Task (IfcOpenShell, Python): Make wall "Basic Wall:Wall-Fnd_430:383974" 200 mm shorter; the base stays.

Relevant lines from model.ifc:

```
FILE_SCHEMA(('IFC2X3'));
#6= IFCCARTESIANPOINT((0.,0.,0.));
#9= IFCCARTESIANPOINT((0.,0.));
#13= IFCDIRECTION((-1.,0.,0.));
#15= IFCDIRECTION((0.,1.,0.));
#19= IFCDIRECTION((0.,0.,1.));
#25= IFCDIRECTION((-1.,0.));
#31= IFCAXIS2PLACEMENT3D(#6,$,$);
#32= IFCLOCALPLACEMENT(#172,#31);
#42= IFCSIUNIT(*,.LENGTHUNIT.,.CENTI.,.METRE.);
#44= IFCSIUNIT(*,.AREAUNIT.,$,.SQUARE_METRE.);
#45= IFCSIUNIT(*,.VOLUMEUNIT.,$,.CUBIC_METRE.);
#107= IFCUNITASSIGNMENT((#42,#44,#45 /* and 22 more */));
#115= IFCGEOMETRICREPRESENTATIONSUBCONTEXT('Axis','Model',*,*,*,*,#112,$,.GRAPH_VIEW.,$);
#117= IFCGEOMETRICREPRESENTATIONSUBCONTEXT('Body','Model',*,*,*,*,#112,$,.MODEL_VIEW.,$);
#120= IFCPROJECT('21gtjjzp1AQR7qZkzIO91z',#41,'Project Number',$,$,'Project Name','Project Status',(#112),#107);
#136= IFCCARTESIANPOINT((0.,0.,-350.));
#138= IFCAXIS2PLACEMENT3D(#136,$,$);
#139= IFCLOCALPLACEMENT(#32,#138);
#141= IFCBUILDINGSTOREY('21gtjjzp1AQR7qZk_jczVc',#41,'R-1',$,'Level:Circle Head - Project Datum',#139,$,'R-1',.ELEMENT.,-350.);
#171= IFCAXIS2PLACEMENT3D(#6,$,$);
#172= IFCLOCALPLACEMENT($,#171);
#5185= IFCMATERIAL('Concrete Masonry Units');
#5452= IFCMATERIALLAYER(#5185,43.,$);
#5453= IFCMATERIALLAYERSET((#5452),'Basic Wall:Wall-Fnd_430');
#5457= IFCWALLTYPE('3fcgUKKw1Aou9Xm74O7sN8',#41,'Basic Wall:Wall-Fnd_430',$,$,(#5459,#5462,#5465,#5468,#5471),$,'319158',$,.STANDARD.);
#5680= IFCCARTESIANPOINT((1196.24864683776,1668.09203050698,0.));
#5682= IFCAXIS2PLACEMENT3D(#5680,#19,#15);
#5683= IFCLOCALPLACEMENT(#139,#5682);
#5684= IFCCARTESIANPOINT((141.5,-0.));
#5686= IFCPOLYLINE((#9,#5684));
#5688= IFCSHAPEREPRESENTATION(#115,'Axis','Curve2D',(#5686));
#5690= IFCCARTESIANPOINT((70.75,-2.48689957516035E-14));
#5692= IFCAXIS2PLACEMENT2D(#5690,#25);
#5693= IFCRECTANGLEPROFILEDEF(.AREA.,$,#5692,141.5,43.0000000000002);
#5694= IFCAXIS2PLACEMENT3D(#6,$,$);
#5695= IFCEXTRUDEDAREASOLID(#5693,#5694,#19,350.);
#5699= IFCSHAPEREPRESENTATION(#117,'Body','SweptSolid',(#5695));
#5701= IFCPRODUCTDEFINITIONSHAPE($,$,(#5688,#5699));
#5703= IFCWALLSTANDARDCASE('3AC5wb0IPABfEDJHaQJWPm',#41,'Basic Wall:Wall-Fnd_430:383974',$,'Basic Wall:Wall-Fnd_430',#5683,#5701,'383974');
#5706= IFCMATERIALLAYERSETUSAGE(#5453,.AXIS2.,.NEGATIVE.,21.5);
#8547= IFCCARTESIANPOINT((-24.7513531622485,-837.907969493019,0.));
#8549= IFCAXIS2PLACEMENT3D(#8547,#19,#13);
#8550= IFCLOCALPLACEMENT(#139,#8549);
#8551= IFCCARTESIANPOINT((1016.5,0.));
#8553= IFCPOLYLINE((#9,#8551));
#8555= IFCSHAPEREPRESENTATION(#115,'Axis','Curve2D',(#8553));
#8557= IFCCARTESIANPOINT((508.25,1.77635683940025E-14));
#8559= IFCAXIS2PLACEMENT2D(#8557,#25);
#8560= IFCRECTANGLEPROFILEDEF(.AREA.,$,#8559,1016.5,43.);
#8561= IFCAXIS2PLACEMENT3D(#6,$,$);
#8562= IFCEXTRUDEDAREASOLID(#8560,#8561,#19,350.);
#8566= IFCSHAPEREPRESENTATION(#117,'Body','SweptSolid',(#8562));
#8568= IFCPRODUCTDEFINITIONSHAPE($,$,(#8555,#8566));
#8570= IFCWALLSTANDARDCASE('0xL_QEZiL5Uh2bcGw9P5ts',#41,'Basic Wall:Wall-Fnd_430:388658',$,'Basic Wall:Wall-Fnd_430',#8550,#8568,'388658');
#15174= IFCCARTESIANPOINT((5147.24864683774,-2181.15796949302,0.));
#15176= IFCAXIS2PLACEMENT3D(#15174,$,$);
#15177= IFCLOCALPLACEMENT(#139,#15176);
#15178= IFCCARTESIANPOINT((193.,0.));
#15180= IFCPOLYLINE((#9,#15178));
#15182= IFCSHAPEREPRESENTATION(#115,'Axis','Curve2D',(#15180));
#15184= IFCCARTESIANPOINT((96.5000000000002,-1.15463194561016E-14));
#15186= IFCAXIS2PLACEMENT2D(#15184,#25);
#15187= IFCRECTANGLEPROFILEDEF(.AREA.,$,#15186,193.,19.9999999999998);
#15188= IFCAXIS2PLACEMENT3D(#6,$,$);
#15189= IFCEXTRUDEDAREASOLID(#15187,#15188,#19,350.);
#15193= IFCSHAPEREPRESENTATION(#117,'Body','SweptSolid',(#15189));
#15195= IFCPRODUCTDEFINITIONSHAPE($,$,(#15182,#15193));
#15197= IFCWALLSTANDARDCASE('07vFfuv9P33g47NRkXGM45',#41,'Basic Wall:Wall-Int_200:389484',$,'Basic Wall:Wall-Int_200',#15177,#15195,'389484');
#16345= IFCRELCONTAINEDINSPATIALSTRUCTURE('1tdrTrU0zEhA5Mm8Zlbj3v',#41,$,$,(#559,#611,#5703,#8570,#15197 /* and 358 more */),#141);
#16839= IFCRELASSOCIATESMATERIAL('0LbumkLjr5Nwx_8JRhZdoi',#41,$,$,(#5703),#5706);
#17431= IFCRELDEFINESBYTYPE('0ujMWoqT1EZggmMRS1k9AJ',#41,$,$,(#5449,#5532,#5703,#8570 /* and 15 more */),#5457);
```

```python
import ifcopenshell
import ifcopenshell.geom
import ifcopenshell.util.representation
import ifcopenshell.util.shape
import ifcopenshell.util.unit

model = ifcopenshell.open("model.ifc")
unit_scale = ifcopenshell.util.unit.calculate_unit_scale(model)
settings = ifcopenshell.geom.settings()


def volume(element):
    """Net volume in cubic metres, openings subtracted."""
    shape = ifcopenshell.geom.create_shape(settings, element)
    return ifcopenshell.util.shape.get_volume(shape.geometry)


wall = model.by_id(5703)
before = volume(wall)

body = ifcopenshell.util.representation.get_representation(wall, "Model", "Body")
solid = body.Items[0]
old_height = solid.Depth
solid.Depth -= 0.2 / unit_scale
after = volume(wall)

print(f"height {old_height:g} -> {solid.Depth:g}, volume {before:.3f} -> {after:.3f} m3")

model.write("model_v2.ifc")
```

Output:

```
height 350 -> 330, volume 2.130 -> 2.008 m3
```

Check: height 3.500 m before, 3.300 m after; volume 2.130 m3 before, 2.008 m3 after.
